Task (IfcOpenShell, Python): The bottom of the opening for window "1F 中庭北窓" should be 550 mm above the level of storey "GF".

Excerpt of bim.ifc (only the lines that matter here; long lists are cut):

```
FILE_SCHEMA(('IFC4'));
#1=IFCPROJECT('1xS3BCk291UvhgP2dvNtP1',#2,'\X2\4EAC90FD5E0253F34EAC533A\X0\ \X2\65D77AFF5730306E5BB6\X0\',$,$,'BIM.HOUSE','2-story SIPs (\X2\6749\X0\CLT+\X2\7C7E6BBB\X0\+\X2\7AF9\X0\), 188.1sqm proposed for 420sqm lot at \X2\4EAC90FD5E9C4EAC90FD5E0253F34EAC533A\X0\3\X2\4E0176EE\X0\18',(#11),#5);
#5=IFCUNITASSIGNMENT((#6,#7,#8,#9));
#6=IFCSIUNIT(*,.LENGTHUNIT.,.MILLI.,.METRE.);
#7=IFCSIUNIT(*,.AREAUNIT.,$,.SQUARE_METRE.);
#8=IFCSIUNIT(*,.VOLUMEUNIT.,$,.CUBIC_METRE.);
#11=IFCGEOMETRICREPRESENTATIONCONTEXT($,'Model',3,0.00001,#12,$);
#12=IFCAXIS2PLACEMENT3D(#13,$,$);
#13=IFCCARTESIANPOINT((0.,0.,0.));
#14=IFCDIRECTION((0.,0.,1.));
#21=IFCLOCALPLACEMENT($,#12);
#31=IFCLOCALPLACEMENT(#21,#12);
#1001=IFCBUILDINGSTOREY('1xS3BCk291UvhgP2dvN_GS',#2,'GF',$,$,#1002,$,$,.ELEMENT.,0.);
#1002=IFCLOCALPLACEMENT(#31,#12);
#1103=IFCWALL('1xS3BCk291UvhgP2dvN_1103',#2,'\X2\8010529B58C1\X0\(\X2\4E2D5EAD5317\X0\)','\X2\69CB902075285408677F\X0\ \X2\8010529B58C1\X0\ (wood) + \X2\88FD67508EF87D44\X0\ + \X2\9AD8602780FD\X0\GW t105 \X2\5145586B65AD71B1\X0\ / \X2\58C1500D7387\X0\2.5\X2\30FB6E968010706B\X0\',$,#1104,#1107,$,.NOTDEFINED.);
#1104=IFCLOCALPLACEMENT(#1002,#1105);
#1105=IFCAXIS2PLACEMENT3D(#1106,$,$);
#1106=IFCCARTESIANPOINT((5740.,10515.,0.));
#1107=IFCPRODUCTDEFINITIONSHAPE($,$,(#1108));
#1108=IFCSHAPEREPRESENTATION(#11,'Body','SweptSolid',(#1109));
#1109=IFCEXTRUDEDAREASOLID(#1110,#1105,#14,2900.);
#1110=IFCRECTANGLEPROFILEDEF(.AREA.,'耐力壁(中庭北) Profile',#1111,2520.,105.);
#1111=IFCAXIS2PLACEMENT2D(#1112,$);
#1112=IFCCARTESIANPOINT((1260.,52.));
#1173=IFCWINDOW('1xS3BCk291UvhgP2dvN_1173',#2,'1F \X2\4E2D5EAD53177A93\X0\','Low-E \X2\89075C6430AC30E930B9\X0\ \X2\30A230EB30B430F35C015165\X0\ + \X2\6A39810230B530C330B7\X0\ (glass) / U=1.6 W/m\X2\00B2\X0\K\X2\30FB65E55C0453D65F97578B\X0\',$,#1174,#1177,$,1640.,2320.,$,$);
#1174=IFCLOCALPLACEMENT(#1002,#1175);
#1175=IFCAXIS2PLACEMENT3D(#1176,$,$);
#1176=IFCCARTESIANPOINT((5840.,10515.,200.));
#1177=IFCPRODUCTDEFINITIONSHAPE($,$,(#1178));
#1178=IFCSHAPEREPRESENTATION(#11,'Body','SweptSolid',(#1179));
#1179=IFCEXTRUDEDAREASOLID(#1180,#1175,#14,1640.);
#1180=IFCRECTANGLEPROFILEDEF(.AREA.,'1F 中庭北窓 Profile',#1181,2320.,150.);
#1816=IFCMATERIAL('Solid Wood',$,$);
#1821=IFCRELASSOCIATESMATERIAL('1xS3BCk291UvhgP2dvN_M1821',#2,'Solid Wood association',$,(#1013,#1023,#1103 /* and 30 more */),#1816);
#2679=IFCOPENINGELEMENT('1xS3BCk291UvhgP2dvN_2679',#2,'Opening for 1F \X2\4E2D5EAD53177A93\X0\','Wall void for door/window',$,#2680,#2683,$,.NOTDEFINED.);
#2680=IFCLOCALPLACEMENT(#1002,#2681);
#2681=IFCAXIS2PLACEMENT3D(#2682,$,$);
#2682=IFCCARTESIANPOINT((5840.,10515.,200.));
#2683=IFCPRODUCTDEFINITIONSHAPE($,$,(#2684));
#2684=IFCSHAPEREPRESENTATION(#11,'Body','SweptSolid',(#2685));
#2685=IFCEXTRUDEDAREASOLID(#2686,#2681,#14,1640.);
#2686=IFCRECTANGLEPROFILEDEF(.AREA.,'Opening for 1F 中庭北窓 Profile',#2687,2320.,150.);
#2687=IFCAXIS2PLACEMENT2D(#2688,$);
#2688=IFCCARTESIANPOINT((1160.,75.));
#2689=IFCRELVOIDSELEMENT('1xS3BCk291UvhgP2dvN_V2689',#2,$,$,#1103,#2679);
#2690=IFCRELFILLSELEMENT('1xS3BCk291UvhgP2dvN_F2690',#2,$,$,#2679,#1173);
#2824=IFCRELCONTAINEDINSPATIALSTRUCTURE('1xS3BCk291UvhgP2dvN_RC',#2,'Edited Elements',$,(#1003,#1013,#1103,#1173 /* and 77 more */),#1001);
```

```python
import numpy as np
import ifcopenshell
import ifcopenshell.api.geometry
import ifcopenshell.geom
import ifcopenshell.util.element
import ifcopenshell.util.placement
import ifcopenshell.util.shape
import ifcopenshell.util.unit

model = ifcopenshell.open("bim.ifc")
unit_scale = ifcopenshell.util.unit.calculate_unit_scale(model)

window = model.by_guid("1xS3BCk291UvhgP2dvN_1173")
opening = window.FillsVoids[0].RelatingOpeningElement
storey = ifcopenshell.util.element.get_container(window, ifc_class="IfcBuildingStorey")
level = ifcopenshell.util.placement.get_local_placement(storey.ObjectPlacement)[2, 3]

# The opening's origin need not be at the sill, so measure its lowest point.
shape = ifcopenshell.geom.create_shape(ifcopenshell.geom.settings(), opening)
bottom = ifcopenshell.util.shape.get_shape_bottom_elevation(shape, shape.geometry) / unit_scale
dz = level + 0.55 / unit_scale - bottom

shift = np.array([0.0, 0.0, dz])
# The window is not placed relative to its opening, so move both.
for product in (opening, window):
    matrix = ifcopenshell.util.placement.get_local_placement(product.ObjectPlacement)
    matrix[:3, 3] += shift
    ifcopenshell.api.geometry.edit_object_placement(model, product=product, matrix=matrix, is_si=False)

print(f"moved by {dz * unit_scale:+.3f} m")

model.write("bim_v2.ifc")
```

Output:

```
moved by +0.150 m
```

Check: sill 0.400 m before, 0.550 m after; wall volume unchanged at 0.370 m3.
